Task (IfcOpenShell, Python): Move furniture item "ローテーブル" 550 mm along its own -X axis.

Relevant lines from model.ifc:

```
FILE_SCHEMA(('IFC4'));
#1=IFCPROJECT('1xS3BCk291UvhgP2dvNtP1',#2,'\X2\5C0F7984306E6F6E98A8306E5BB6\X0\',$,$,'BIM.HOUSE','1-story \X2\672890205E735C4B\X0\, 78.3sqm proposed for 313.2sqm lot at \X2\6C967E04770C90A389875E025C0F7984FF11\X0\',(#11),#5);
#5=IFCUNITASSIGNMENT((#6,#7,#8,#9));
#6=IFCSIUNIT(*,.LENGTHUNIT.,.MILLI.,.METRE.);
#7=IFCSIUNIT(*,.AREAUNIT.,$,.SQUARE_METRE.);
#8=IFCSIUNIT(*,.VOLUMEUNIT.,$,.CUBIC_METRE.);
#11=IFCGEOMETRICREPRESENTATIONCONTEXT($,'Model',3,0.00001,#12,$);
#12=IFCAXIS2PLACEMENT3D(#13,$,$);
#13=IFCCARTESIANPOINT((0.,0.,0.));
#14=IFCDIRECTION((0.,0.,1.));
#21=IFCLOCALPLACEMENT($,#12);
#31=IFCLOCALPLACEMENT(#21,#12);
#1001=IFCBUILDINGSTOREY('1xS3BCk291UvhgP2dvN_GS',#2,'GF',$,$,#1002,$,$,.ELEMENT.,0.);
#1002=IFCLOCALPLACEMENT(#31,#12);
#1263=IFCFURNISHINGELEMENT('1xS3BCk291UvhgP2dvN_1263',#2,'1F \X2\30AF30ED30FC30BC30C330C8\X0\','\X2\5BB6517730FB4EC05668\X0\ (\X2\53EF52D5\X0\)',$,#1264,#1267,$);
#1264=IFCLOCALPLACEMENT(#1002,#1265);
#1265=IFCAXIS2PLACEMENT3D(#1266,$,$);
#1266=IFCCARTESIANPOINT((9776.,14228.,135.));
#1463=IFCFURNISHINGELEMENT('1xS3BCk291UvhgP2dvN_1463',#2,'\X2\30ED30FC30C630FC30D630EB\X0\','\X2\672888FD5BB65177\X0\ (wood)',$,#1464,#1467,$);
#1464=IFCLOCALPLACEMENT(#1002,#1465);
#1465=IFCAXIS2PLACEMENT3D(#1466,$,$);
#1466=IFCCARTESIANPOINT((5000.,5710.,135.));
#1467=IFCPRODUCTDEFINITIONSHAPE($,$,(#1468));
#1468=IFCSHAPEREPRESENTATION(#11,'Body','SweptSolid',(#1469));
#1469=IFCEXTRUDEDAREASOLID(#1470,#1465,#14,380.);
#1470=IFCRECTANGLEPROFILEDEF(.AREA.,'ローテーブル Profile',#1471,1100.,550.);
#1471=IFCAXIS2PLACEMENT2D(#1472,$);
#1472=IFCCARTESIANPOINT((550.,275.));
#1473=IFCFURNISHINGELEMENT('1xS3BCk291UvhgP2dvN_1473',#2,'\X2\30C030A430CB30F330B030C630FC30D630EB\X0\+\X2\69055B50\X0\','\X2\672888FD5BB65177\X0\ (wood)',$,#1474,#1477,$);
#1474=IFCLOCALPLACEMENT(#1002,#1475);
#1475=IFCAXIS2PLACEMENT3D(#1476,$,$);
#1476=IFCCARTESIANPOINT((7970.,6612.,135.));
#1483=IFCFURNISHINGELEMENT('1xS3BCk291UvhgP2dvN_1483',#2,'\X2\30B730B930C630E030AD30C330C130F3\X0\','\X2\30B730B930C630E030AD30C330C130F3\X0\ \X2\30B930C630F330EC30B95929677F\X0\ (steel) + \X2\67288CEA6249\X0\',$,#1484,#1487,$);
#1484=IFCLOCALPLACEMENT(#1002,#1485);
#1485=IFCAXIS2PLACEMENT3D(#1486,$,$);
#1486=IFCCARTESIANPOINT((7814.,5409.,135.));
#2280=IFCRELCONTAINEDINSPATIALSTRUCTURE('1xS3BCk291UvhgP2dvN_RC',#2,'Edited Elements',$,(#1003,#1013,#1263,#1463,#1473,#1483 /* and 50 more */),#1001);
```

```python
import ifcopenshell
import ifcopenshell.api.geometry
import ifcopenshell.util.placement

model = ifcopenshell.open("model.ifc")

item = model.by_guid("1xS3BCk291UvhgP2dvN_1463")
matrix = ifcopenshell.util.placement.get_local_placement(item.ObjectPlacement)
matrix[:3, 3] -= matrix[:3, 0] * 550.0
ifcopenshell.api.geometry.edit_object_placement(model, product=item, matrix=matrix, is_si=False)

print(ifcopenshell.util.placement.get_local_placement(item.ObjectPlacement).round(3) + 0.0)

model.write("model_v2.ifc")
```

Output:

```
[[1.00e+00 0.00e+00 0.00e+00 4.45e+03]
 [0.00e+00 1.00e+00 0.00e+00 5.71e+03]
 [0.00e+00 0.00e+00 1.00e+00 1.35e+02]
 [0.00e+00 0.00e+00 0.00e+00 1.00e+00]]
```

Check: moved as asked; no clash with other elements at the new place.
